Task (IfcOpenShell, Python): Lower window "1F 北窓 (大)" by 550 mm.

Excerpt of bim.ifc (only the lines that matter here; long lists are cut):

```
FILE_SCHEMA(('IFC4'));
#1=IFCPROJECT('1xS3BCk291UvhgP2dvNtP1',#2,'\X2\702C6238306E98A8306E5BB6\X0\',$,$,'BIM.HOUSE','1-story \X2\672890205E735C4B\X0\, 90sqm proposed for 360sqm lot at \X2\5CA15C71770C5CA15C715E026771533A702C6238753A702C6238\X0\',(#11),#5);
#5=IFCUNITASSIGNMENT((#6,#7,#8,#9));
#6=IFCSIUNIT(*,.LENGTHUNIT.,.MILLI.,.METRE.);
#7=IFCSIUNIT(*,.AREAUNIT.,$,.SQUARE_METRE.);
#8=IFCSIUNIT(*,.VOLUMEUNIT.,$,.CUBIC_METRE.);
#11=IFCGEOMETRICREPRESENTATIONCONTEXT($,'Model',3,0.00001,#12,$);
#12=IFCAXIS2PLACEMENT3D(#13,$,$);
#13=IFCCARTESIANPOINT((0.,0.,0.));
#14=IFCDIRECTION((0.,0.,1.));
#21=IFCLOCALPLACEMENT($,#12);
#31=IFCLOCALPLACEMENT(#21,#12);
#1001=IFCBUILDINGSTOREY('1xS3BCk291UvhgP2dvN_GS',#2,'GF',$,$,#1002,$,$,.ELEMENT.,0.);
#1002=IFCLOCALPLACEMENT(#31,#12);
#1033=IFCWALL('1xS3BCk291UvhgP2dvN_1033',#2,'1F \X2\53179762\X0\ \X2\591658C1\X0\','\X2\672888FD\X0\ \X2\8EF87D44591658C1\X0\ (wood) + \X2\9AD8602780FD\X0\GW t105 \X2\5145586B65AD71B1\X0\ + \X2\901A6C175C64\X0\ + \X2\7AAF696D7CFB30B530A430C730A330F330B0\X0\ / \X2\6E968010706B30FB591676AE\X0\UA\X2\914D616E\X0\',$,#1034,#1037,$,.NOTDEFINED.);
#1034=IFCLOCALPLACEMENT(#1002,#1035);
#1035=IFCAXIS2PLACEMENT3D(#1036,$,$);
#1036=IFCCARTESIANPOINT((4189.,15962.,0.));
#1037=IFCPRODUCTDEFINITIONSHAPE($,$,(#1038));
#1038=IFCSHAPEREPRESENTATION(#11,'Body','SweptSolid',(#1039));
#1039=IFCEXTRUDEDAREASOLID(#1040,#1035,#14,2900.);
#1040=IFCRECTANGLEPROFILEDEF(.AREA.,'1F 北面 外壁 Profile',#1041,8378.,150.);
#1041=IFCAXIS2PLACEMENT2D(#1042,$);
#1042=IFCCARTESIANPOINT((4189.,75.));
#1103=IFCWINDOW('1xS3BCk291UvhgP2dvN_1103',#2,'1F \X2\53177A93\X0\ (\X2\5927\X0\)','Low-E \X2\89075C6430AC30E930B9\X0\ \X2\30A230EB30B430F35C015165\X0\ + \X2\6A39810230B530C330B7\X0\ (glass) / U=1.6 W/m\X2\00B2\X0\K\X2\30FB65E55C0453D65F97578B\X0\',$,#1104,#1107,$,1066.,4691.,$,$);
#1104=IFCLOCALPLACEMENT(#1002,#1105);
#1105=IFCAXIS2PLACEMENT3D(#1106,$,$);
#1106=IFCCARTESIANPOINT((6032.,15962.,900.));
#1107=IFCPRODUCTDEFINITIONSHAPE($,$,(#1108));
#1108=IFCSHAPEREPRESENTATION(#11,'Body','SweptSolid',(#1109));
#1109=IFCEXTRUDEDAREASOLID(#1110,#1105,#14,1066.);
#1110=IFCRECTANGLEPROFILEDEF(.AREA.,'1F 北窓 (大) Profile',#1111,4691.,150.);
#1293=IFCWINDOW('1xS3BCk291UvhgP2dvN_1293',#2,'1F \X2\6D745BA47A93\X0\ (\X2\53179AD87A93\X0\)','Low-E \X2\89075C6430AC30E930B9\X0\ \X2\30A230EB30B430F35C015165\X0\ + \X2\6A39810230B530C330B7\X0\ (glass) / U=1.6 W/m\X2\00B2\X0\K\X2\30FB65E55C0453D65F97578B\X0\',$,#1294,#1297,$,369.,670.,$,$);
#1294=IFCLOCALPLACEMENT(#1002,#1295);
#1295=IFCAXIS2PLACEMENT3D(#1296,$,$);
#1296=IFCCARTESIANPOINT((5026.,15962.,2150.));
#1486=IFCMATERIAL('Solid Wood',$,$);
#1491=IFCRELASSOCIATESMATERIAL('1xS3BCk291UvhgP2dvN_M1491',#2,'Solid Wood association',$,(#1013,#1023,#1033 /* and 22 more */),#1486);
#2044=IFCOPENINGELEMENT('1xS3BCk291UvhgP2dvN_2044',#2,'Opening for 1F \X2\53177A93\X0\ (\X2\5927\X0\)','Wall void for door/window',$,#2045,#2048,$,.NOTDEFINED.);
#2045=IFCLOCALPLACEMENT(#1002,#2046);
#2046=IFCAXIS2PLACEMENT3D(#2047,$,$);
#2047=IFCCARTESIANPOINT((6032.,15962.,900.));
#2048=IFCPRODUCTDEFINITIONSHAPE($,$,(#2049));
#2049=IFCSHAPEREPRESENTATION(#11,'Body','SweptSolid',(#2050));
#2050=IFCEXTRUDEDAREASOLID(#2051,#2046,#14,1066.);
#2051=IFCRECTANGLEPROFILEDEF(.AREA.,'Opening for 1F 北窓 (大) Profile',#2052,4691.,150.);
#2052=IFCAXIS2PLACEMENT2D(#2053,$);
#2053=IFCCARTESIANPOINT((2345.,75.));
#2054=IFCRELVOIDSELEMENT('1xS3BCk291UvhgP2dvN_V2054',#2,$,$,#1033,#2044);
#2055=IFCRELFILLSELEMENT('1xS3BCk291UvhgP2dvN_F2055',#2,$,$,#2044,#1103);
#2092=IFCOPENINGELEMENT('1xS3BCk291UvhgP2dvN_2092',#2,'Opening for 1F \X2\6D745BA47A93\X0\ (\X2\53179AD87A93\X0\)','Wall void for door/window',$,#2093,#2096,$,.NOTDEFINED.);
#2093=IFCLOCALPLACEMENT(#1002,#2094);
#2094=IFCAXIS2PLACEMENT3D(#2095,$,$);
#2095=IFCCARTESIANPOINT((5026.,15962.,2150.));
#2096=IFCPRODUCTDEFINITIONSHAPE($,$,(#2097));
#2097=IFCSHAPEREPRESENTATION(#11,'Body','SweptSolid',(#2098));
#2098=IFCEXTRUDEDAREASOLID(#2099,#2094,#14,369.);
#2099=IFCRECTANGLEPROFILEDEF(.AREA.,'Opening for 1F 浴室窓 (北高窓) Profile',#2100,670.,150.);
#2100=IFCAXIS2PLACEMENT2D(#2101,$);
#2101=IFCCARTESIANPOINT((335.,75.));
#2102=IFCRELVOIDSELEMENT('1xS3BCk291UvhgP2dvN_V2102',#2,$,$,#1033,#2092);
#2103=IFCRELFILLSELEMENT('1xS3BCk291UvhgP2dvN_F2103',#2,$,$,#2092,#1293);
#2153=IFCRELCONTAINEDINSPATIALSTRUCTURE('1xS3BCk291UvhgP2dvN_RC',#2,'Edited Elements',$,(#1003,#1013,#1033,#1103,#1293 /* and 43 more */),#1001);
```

```python
import numpy as np
import ifcopenshell
import ifcopenshell.api.geometry
import ifcopenshell.util.placement
import ifcopenshell.util.unit

model = ifcopenshell.open("bim.ifc")
unit_scale = ifcopenshell.util.unit.calculate_unit_scale(model)

window = model.by_guid("1xS3BCk291UvhgP2dvN_1103")
opening = window.FillsVoids[0].RelatingOpeningElement
dz = -550.0

shift = np.array([0.0, 0.0, dz])
# The window is not placed relative to its opening, so move both.
for product in (opening, window):
    matrix = ifcopenshell.util.placement.get_local_placement(product.ObjectPlacement)
    matrix[:3, 3] += shift
    ifcopenshell.api.geometry.edit_object_placement(model, product=product, matrix=matrix, is_si=False)

print(f"moved by {dz * unit_scale:+.3f} m")

model.write("bim_v2.ifc")
```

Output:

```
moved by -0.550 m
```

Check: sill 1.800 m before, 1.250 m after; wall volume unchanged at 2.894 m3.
